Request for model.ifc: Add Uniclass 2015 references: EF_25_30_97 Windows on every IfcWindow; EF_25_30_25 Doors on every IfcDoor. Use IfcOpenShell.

First a look at what the model holds.

```python
import ifcopenshell

model = ifcopenshell.open("model.ifc")
print(model.schema)
print("classifications:", [c.Name for c in model.by_type("IfcClassification")])
for ifc_class in ("IfcDoor", "IfcRoof", "IfcStair", "IfcWall", "IfcWindow"):
    print(ifc_class, len(model.by_type(ifc_class)))
```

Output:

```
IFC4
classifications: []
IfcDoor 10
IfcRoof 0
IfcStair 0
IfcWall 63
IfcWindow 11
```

```python
import ifcopenshell
import ifcopenshell.api.classification

model = ifcopenshell.open("model.ifc")

system = ifcopenshell.api.classification.add_classification(model, classification="Uniclass 2015")

codes = {
    "IfcWindow": ("EF_25_30_97", "Windows"),
    "IfcDoor": ("EF_25_30_25", "Doors"),
}
for ifc_class, (code, name) in codes.items():
    products = model.by_type(ifc_class)
    ifcopenshell.api.classification.add_reference(
        model, products=products, classification=system, identification=code, name=name
    )
    print(code, len(products))

model.write("model_updated.ifc")
```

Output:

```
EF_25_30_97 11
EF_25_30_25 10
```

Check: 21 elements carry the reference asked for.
